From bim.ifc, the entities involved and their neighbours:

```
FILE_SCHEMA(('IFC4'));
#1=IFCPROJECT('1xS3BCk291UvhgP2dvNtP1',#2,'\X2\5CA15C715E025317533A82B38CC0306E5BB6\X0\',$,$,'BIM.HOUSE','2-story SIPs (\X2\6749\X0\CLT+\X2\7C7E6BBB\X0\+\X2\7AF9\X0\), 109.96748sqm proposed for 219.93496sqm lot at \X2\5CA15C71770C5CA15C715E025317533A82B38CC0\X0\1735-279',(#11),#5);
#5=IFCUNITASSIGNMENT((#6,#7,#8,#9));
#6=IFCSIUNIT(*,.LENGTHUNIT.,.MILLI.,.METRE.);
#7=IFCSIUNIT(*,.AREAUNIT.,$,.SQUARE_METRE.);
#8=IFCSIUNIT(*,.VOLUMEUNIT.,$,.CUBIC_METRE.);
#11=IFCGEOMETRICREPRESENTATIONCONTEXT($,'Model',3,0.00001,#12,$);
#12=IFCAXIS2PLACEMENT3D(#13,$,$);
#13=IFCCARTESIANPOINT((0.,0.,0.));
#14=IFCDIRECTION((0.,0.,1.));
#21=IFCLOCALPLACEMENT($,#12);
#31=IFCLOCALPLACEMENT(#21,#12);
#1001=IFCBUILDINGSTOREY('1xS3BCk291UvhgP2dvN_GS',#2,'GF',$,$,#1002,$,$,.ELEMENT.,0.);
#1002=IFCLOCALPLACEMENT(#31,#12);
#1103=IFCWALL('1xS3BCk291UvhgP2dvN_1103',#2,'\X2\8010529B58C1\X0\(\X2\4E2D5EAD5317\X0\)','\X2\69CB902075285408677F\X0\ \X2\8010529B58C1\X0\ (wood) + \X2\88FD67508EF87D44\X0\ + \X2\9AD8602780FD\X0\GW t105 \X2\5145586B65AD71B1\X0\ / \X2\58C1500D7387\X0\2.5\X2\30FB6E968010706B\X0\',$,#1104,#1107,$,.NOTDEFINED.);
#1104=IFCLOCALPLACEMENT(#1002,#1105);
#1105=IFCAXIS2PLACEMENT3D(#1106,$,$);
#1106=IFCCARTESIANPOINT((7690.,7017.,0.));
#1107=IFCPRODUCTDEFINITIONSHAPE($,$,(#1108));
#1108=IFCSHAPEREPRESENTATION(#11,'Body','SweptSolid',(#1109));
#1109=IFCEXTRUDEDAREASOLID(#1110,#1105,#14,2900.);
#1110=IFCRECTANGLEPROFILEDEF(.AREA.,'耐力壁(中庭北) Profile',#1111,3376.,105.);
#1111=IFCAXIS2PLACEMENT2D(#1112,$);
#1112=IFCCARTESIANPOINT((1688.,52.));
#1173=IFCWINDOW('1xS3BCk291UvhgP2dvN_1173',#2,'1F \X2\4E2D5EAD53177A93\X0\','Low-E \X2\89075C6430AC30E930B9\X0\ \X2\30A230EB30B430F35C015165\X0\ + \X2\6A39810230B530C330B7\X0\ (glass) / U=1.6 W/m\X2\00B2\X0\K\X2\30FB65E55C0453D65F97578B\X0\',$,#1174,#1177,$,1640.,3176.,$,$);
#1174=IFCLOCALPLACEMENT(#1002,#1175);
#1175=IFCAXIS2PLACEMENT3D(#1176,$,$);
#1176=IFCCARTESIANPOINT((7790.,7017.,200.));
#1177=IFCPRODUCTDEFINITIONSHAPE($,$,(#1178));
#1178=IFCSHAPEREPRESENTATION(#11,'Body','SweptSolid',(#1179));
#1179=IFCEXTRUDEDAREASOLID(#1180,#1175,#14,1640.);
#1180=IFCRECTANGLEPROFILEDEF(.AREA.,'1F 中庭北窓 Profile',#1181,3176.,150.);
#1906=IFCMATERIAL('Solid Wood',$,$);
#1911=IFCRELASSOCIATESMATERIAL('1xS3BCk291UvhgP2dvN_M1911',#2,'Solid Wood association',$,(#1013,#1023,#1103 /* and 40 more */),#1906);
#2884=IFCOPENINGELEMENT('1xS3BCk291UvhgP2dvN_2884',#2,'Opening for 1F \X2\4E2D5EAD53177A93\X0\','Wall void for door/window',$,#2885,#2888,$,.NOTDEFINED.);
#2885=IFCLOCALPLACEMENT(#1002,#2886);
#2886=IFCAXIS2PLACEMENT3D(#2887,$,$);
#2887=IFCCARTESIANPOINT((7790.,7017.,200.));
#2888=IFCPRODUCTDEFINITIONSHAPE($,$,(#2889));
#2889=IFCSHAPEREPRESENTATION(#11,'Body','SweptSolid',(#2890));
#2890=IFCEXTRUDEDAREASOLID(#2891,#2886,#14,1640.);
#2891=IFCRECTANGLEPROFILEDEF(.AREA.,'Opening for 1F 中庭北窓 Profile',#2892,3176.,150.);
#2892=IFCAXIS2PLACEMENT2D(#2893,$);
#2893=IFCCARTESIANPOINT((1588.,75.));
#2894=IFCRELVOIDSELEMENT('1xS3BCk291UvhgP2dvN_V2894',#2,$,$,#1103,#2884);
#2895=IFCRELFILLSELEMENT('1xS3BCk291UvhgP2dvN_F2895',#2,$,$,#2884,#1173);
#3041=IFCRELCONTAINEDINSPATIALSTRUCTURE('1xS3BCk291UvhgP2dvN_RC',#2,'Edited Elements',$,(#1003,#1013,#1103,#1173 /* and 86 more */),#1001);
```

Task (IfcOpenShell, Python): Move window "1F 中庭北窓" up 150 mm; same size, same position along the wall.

```python
import numpy as np
import ifcopenshell
import ifcopenshell.api.geometry
import ifcopenshell.util.placement
import ifcopenshell.util.unit

model = ifcopenshell.open("bim.ifc")
unit_scale = ifcopenshell.util.unit.calculate_unit_scale(model)

window = model.by_guid("1xS3BCk291UvhgP2dvN_1173")
opening = window.FillsVoids[0].RelatingOpeningElement
dz = 0.15 / unit_scale

shift = np.array([0.0, 0.0, dz])
# The window is not placed relative to its opening, so move both.
for product in (opening, window):
    matrix = ifcopenshell.util.placement.get_local_placement(product.ObjectPlacement)
    matrix[:3, 3] += shift
    ifcopenshell.api.geometry.edit_object_placement(model, product=product, matrix=matrix, is_si=False)

print(f"moved by {dz * unit_scale:+.3f} m")

model.write("bim_v2.ifc")
```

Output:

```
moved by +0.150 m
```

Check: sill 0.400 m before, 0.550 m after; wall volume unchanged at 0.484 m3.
